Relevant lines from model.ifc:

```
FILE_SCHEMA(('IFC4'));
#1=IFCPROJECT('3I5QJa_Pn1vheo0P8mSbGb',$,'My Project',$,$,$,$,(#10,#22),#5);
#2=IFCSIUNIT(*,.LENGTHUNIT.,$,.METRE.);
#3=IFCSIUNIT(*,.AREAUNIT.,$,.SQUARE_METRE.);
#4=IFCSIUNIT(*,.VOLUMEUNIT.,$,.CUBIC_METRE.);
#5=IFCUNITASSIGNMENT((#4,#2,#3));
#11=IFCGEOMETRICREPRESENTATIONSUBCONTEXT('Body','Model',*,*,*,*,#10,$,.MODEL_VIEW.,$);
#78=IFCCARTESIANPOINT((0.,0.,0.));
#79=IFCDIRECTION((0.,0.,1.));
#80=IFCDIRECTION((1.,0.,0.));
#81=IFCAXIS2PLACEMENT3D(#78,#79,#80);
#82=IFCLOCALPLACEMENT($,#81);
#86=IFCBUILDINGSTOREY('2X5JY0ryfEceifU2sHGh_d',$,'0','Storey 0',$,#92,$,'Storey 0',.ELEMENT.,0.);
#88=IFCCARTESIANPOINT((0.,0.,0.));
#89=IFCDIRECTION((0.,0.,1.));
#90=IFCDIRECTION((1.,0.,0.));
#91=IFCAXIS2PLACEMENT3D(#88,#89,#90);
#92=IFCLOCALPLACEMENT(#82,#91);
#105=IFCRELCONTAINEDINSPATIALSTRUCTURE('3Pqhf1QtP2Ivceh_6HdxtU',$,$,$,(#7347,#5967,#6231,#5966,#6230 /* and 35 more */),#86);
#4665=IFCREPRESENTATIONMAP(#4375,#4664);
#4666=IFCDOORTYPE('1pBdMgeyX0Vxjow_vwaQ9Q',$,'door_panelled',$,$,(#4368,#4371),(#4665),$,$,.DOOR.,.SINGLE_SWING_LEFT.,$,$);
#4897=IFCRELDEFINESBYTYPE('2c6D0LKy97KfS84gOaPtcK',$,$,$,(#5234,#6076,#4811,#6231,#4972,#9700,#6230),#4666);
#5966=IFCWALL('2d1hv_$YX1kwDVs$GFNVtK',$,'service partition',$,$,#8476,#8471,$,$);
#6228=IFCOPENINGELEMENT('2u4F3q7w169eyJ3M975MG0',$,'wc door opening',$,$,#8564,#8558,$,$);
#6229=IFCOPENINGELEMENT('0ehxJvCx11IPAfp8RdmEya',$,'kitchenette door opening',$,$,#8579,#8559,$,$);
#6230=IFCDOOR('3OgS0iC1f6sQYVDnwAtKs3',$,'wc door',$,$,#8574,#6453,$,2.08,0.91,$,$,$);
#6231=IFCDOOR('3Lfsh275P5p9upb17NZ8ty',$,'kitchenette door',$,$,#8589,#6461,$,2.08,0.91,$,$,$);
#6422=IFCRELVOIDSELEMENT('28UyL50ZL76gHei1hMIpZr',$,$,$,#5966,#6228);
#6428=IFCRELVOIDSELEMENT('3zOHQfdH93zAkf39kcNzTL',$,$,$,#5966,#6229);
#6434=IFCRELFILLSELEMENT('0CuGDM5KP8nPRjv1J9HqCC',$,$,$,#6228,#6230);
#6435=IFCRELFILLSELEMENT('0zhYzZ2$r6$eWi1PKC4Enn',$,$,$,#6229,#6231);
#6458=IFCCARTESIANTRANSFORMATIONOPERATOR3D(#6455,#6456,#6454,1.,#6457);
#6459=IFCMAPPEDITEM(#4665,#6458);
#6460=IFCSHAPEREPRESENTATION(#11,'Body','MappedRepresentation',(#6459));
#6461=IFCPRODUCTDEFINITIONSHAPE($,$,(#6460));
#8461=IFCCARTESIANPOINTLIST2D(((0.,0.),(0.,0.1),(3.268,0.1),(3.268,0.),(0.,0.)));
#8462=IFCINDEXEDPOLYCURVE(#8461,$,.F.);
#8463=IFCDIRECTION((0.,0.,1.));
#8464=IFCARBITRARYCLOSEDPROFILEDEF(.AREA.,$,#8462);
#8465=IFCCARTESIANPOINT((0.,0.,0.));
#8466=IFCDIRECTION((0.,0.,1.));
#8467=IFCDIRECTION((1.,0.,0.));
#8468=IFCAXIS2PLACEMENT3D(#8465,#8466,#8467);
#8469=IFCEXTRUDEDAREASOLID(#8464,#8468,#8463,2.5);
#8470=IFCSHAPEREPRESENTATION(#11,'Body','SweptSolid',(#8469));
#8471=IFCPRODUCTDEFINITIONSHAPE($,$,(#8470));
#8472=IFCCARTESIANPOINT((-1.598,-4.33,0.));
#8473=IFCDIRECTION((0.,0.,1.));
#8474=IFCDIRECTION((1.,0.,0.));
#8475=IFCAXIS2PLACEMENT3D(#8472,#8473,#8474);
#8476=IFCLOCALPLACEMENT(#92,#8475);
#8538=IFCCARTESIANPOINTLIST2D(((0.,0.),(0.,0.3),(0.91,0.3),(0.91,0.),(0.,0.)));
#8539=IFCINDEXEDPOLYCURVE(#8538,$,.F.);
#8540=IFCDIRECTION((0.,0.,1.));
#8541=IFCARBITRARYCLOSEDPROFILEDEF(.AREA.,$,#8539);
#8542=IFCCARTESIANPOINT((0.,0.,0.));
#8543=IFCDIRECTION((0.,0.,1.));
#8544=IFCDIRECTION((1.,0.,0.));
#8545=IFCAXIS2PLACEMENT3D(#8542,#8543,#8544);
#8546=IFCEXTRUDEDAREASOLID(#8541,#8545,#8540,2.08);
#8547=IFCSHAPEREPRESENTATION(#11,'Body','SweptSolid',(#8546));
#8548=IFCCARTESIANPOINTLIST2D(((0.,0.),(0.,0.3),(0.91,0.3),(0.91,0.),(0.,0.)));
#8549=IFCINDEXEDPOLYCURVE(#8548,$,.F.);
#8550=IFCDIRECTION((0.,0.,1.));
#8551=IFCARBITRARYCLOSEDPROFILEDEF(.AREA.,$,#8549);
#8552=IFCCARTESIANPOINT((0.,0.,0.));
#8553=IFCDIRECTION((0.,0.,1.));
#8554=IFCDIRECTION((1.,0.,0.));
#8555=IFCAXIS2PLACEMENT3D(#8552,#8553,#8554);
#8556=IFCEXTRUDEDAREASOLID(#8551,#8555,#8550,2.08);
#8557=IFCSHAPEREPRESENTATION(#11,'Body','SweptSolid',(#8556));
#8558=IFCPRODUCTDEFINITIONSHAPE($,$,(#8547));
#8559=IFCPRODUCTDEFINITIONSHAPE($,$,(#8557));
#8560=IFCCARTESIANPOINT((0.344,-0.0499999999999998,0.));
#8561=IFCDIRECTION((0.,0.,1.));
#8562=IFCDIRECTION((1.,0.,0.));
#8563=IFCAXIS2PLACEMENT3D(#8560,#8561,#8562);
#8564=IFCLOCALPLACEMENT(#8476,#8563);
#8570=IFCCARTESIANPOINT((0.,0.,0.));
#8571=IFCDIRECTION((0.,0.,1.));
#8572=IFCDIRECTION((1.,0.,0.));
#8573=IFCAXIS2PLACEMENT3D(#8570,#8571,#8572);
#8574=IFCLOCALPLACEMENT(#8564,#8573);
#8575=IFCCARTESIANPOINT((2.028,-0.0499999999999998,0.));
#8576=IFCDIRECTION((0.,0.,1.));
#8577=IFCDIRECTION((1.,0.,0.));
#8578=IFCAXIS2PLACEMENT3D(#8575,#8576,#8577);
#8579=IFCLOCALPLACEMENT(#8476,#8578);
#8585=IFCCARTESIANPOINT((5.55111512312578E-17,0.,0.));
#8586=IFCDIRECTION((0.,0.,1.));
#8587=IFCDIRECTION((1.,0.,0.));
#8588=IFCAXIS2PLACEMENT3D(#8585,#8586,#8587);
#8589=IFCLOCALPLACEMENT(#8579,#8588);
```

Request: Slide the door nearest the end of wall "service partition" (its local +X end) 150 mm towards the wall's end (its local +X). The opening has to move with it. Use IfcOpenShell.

```python
import ifcopenshell
import ifcopenshell.api.geometry
import ifcopenshell.util.placement

model = ifcopenshell.open("model.ifc")

door = model.by_id(6231)
opening = door.FillsVoids[0].RelatingOpeningElement
wall = opening.VoidsElements[0].RelatingBuildingElement

wall_matrix = ifcopenshell.util.placement.get_local_placement(wall.ObjectPlacement)
shift = wall_matrix[:3, 0] * 0.15
before = ifcopenshell.util.placement.get_local_placement(door.ObjectPlacement)[:3, 3].copy()

# The door is placed relative to its opening, so it follows when the opening moves.
matrix = ifcopenshell.util.placement.get_local_placement(opening.ObjectPlacement)
matrix[:3, 3] += shift
ifcopenshell.api.geometry.edit_object_placement(
    model, product=opening, matrix=matrix, is_si=False, should_transform_children=True
)

after = ifcopenshell.util.placement.get_local_placement(door.ObjectPlacement)[:3, 3]
print("door moved by", (after - before).round(3) + 0.0)

model.write("model_v2.ifc")
```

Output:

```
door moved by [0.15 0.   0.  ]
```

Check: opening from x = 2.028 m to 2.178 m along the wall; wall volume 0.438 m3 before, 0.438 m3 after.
